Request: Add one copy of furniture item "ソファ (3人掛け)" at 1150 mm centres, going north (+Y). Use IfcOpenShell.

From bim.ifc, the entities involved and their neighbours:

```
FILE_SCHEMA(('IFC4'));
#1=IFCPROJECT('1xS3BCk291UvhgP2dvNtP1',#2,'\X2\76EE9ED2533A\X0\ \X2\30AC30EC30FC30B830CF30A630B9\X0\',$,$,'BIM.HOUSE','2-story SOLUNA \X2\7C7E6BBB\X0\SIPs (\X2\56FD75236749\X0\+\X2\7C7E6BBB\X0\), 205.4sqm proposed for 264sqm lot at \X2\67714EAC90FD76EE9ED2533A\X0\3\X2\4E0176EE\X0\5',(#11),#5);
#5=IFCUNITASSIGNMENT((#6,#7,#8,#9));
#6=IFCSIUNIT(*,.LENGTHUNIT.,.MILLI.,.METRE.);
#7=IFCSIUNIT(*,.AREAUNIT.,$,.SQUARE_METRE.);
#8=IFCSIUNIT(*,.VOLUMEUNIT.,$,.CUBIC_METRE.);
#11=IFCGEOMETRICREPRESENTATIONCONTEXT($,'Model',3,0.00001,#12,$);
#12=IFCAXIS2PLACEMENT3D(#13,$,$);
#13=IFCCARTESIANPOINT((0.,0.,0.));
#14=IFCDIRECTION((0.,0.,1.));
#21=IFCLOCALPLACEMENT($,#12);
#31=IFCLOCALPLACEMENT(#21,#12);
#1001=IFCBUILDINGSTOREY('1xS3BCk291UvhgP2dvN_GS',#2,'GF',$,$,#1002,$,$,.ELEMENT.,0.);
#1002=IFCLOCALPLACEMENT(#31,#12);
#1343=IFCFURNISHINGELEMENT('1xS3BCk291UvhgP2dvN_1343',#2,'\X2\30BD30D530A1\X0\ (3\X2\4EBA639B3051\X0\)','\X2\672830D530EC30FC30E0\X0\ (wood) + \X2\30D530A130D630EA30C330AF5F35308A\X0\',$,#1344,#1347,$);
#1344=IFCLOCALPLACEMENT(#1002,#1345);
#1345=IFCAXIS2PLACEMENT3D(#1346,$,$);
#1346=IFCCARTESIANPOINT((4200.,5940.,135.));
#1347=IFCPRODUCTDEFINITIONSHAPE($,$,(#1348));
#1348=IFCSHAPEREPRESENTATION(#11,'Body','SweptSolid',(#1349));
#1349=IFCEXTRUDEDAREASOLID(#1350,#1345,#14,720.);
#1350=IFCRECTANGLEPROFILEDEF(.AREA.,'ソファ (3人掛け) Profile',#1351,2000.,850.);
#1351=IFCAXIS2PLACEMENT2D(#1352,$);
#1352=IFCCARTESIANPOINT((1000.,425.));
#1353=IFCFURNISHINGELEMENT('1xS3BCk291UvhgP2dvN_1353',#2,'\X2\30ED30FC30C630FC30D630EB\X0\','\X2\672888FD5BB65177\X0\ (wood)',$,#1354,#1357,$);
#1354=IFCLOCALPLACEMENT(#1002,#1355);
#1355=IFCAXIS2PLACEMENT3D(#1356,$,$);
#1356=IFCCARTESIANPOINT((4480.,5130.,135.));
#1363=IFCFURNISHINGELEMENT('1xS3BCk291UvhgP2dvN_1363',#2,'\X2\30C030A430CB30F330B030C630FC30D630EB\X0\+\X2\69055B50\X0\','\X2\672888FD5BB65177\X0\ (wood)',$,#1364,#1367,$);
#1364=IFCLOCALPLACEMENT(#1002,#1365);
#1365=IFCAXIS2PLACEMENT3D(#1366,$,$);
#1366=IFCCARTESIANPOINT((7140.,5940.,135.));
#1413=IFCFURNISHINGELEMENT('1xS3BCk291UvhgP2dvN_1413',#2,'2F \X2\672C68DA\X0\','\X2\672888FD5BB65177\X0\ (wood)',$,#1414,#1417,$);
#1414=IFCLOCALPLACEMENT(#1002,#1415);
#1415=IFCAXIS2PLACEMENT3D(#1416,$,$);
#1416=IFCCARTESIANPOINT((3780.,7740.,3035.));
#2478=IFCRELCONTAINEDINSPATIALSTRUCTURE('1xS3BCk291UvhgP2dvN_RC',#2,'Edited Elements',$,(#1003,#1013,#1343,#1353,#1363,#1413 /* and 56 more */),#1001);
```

```python
import numpy as np
import ifcopenshell
import ifcopenshell.api.geometry
import ifcopenshell.api.root
import ifcopenshell.util.element
import ifcopenshell.util.placement
import ifcopenshell.util.unit

model = ifcopenshell.open("bim.ifc")
unit_scale = ifcopenshell.util.unit.calculate_unit_scale(model)


def reuse_history(source, copy):
    """copy_class also copies each property set's owner history, people and application; keep the originals."""
    for rel in copy.IsDefinedBy:
        if rel.is_a("IfcRelDefinesByProperties") and (history := rel.RelatingPropertyDefinition.OwnerHistory):
            rel.RelatingPropertyDefinition.OwnerHistory = source.OwnerHistory
            ifcopenshell.util.element.remove_deep2(model, history)


source = model.by_guid("1xS3BCk291UvhgP2dvN_1343")
base = ifcopenshell.util.placement.get_local_placement(source.ObjectPlacement)
step = np.array([0.0, 1.0, 0.0]) * 1.15 / unit_scale

for i in range(1, 2):
    copy = ifcopenshell.api.root.copy_class(model, product=source)
    copy.Representation = ifcopenshell.util.element.copy_deep(
        model, source.Representation, exclude=["IfcGeometricRepresentationContext", "IfcRepresentationMap"]
    )
    reuse_history(source, copy)
    matrix = base.copy()
    matrix[:3, 3] += i * step
    print("added at", matrix[:3, 3].round(3) + 0.0)
    ifcopenshell.api.geometry.edit_object_placement(model, product=copy, matrix=matrix, is_si=False)

model.write("bim_v2.ifc")
```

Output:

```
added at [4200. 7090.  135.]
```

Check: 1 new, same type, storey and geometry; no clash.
